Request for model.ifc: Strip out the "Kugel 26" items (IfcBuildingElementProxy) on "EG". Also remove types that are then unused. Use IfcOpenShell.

First a look at what the model holds.

```python
import ifcopenshell
import ifcopenshell.util.element

model = ifcopenshell.open("model.ifc")
print(model.schema)
storey = next(s for s in model.by_type("IfcBuildingStorey") if s.Name == "EG")
proxies = [e for e in ifcopenshell.util.element.get_decomposition(storey) if e.is_a("IfcBuildingElementProxy")]
seen = {}
for e in proxies:
    element_type = ifcopenshell.util.element.get_type(e)
    name = element_type.Name if element_type not in (None, e) else None
    seen[name] = seen.get(name, 0) + 1
for name, count in sorted(seen.items(), key=str):
    print(count, "x", name)
```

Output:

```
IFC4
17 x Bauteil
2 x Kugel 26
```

```python
import ifcopenshell
import ifcopenshell.api.root
import ifcopenshell.util.element

model = ifcopenshell.open("model.ifc")

storey = next(s for s in model.by_type("IfcBuildingStorey") if s.Name == "EG")
proxies = [e for e in ifcopenshell.util.element.get_decomposition(storey) if e.is_a("IfcBuildingElementProxy")]
targets = [e for e in proxies if (t := ifcopenshell.util.element.get_type(e)) not in (None, e) and t.Name == "Kugel 26"]
types = {ifcopenshell.util.element.get_type(e) for e in targets} - {None, *targets}

for e in targets:
    ifcopenshell.api.root.remove_product(model, product=e)
print(len(targets), "removed")

unused = [t for t in types if not ifcopenshell.util.element.get_types(t)]
for t in unused:
    ifcopenshell.api.root.remove_product(model, product=t)
print(len(unused), "unused types removed")

model.write("model_edited.ifc")
```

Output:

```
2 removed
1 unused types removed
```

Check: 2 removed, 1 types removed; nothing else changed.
